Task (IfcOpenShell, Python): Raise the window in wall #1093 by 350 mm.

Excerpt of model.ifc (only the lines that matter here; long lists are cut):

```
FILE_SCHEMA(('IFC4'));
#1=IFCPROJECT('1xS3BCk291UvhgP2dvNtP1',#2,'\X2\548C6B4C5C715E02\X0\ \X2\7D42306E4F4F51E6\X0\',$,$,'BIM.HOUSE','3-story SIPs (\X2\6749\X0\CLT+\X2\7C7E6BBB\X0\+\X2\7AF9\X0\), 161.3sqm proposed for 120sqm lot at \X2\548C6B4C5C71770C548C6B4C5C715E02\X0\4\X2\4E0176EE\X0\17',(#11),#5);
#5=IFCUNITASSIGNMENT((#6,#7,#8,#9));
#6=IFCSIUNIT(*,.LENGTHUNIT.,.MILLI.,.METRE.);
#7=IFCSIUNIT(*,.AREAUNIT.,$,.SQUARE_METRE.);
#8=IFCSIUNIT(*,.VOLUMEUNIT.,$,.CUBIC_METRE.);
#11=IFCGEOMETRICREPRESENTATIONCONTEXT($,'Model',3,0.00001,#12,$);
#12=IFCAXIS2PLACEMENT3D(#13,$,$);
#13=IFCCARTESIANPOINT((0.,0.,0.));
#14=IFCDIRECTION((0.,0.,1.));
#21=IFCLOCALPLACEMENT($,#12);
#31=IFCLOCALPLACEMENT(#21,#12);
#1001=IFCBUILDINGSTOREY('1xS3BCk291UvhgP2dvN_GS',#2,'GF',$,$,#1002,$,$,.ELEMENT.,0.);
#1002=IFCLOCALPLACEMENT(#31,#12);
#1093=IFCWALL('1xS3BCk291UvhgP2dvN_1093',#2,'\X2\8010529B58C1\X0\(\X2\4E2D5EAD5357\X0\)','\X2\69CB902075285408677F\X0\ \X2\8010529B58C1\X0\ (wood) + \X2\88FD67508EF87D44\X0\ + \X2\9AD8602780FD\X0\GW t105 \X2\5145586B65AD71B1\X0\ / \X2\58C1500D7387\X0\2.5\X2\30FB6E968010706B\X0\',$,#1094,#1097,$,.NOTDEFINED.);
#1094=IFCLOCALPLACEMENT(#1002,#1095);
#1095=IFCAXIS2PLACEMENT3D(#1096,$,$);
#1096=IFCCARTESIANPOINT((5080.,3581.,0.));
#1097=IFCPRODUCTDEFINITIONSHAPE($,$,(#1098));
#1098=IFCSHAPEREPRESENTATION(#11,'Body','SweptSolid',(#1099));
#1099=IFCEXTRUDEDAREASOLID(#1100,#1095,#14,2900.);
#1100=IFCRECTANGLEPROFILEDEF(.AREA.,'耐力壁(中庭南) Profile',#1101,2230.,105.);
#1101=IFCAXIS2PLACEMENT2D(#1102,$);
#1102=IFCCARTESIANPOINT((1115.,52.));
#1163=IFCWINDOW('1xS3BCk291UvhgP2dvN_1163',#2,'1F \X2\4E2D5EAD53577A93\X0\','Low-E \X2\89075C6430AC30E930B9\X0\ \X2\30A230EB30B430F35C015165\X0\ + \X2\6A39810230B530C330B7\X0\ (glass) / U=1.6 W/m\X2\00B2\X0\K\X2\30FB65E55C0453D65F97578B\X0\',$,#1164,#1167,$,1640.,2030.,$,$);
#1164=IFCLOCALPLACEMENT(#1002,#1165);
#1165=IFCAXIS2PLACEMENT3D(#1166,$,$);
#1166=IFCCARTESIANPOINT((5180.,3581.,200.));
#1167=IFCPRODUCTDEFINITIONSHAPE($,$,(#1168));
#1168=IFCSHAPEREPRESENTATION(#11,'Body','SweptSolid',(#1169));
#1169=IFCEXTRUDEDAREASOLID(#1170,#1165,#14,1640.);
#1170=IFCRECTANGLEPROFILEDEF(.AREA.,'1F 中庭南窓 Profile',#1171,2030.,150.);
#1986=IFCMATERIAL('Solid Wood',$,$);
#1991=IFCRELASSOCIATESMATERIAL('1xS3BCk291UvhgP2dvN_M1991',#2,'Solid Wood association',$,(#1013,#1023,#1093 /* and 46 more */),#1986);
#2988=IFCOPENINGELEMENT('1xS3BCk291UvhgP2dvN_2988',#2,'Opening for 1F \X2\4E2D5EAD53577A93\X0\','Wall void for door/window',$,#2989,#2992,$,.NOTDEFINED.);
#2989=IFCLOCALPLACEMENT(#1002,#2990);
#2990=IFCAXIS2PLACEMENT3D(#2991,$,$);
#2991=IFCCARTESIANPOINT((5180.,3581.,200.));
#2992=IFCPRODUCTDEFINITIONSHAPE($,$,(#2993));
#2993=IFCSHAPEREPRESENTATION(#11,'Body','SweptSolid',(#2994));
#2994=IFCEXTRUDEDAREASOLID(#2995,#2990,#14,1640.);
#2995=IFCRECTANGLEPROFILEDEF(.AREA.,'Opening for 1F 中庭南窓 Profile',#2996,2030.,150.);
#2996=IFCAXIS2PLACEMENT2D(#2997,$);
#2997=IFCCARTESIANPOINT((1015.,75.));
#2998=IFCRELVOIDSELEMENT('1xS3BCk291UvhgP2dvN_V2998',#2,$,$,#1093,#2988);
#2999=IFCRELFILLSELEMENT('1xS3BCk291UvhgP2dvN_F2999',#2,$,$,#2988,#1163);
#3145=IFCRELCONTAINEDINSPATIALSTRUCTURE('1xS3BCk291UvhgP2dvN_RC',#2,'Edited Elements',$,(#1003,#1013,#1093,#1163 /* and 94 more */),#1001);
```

```python
import numpy as np
import ifcopenshell
import ifcopenshell.api.geometry
import ifcopenshell.util.placement
import ifcopenshell.util.unit

model = ifcopenshell.open("model.ifc")
unit_scale = ifcopenshell.util.unit.calculate_unit_scale(model)

window = model.by_guid("1xS3BCk291UvhgP2dvN_1163")
opening = window.FillsVoids[0].RelatingOpeningElement
dz = 0.35 / unit_scale

shift = np.array([0.0, 0.0, dz])
# The window is not placed relative to its opening, so move both.
for product in (opening, window):
    matrix = ifcopenshell.util.placement.get_local_placement(product.ObjectPlacement)
    matrix[:3, 3] += shift
    ifcopenshell.api.geometry.edit_object_placement(model, product=product, matrix=matrix, is_si=False)

print(f"moved by {dz * unit_scale:+.3f} m")

model.write("model-out.ifc")
```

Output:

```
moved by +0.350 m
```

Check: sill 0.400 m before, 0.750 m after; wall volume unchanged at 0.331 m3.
